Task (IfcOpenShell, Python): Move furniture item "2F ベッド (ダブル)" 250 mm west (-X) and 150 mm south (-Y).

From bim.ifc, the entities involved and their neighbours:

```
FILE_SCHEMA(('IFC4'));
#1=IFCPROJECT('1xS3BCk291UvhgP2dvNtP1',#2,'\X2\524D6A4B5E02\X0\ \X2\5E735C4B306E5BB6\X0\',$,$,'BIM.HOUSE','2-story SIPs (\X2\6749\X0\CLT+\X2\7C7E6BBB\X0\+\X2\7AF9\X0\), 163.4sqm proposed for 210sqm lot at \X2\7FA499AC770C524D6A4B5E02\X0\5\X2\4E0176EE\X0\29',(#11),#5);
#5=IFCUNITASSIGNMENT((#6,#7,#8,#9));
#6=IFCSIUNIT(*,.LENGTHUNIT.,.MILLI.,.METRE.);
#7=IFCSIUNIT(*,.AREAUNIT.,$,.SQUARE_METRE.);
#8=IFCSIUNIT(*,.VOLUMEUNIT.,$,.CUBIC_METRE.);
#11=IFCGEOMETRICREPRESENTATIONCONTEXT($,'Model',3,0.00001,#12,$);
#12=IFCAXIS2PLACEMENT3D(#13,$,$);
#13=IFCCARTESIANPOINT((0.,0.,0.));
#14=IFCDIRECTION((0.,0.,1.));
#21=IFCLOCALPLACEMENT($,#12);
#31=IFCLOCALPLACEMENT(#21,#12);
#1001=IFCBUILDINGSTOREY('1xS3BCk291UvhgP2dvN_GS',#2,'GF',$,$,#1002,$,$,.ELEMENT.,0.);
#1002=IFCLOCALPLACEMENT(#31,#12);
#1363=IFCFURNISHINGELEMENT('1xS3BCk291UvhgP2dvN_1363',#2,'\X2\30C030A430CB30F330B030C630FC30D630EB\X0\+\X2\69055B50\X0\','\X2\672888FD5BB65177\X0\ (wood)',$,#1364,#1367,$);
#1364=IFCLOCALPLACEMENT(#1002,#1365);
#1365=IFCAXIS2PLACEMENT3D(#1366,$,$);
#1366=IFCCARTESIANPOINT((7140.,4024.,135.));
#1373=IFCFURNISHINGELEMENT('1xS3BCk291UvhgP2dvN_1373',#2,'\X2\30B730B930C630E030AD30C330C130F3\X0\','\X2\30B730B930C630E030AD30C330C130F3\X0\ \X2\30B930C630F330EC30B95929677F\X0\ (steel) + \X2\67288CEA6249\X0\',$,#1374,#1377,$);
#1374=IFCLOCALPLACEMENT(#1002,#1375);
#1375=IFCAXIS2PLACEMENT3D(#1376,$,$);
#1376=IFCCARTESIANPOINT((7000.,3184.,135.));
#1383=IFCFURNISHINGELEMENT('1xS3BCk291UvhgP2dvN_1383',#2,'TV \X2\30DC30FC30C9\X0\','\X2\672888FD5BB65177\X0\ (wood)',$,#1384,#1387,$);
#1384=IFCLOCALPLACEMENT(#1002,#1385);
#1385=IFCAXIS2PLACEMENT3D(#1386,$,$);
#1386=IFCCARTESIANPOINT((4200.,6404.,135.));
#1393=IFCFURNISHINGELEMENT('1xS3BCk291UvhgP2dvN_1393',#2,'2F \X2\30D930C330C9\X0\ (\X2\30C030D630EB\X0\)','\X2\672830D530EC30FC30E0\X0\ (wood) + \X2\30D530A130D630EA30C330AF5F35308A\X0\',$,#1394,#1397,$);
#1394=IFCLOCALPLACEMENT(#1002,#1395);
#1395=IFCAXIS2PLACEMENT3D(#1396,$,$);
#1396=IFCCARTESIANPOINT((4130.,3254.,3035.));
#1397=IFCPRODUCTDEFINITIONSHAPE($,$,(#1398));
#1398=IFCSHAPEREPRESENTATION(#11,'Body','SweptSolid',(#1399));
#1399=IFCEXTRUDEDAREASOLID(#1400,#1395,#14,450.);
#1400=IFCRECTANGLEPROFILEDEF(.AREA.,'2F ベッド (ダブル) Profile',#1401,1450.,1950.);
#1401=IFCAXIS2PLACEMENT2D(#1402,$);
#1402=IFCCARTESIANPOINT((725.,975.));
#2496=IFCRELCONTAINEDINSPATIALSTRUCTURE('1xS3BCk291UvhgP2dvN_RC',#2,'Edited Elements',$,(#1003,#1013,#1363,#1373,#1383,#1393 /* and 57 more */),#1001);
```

```python
import ifcopenshell
import ifcopenshell.api.geometry
import ifcopenshell.util.placement

model = ifcopenshell.open("bim.ifc")

item = model.by_guid("1xS3BCk291UvhgP2dvN_1393")
matrix = ifcopenshell.util.placement.get_local_placement(item.ObjectPlacement)
matrix[0, 3] -= 250.0
matrix[1, 3] -= 150.0
ifcopenshell.api.geometry.edit_object_placement(model, product=item, matrix=matrix, is_si=False)

print(ifcopenshell.util.placement.get_local_placement(item.ObjectPlacement).round(3) + 0.0)

model.write("bim_v2.ifc")
```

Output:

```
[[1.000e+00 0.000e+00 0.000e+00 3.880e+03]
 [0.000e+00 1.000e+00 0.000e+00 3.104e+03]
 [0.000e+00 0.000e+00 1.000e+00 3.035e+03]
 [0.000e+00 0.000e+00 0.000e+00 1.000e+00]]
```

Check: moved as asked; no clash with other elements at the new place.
